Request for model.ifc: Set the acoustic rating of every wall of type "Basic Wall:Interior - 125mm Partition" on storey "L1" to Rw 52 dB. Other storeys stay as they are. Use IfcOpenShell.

First a look at what the model holds.

```python
import ifcopenshell
import ifcopenshell.util.element

model = ifcopenshell.open("model.ifc")
print(model.schema)
storey = next(s for s in model.by_type("IfcBuildingStorey") if s.Name == "L1")
walls = [e for e in ifcopenshell.util.element.get_decomposition(storey) if e.is_a("IfcWall")]
seen = {}
for e in walls:
    element_type = ifcopenshell.util.element.get_type(e)
    key = (element_type.Name if element_type != e and element_type else None, ifcopenshell.util.element.get_pset(e, "Pset_WallCommon", "AcousticRating"))
    seen[key] = seen.get(key, 0) + 1
for (name, value), count in sorted(seen.items(), key=str):
    print(count, "x", name, "|", value)
```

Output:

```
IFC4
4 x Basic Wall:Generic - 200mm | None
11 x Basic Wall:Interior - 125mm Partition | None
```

```python
import ifcopenshell
import ifcopenshell.api.pset
import ifcopenshell.util.element

model = ifcopenshell.open("model.ifc")

storey = next(s for s in model.by_type("IfcBuildingStorey") if s.Name == "L1")
walls = [e for e in ifcopenshell.util.element.get_decomposition(storey) if e.is_a("IfcWall")]

count = 0
for e in walls:
    element_type = ifcopenshell.util.element.get_type(e)
    if element_type in (None, e) or element_type.Name != "Basic Wall:Interior - 125mm Partition":
        continue
    # add_pset returns the element's existing set when there is one.
    pset = ifcopenshell.api.pset.add_pset(model, product=e, name="Pset_WallCommon")
    ifcopenshell.api.pset.edit_pset(model, pset=pset, properties={"AcousticRating": "Rw 52 dB"})
    count += 1

print(count, "walls updated")

model.write("model_updated.ifc")
```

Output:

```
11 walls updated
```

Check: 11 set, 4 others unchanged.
